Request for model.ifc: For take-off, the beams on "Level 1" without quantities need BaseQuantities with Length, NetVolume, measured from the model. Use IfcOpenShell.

First a look at what the model holds.

```python
import ifcopenshell
import ifcopenshell.util.element
import ifcopenshell.util.unit

model = ifcopenshell.open("model.ifc")
print(model.schema)
for unit_type in ("LENGTHUNIT", "AREAUNIT", "VOLUMEUNIT"):
    print(unit_type, ifcopenshell.util.unit.calculate_unit_scale(model, unit_type))
storey = next(s for s in model.by_type("IfcBuildingStorey") if s.Name == "Level 1")
beams = [e for e in ifcopenshell.util.element.get_decomposition(storey) if e.is_a("IfcBeam")]
for e in sorted(beams, key=lambda e: e.id()):
    print(e.id(), e.is_a(), e.Name, list(ifcopenshell.util.element.get_psets(e, qtos_only=True)), sep=" | ")
```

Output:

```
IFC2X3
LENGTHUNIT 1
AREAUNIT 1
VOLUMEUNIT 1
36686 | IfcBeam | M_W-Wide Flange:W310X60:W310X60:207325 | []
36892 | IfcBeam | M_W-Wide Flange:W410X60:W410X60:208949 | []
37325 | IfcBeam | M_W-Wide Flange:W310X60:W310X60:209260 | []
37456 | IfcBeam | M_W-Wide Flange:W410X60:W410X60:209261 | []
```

```python
import ifcopenshell
import ifcopenshell.api.pset
import ifcopenshell.geom
import ifcopenshell.util.element
import ifcopenshell.util.shape
import ifcopenshell.util.unit

model = ifcopenshell.open("model.ifc")
unit_scale = ifcopenshell.util.unit.calculate_unit_scale(model)
volume_scale = ifcopenshell.util.unit.calculate_unit_scale(model, "VOLUMEUNIT")
settings = ifcopenshell.geom.settings()

storey = next(s for s in model.by_type("IfcBuildingStorey") if s.Name == "Level 1")
beams = [e for e in ifcopenshell.util.element.get_decomposition(storey) if e.is_a("IfcBeam")]

for e in sorted(beams, key=lambda e: e.id()):
    if ifcopenshell.util.element.get_psets(e, qtos_only=True, should_inherit=False):
        continue
    # Geometry comes back in metres, in the element's own axes.
    shape = ifcopenshell.geom.create_shape(settings, e)
    values = {
        "Length": ifcopenshell.util.shape.get_max_xyz(shape.geometry) / unit_scale,
        "NetVolume": ifcopenshell.util.shape.get_volume(shape.geometry) / volume_scale,
    }
    qto = ifcopenshell.api.pset.add_qto(model, product=e, name="BaseQuantities")
    ifcopenshell.api.pset.edit_qto(model, qto=qto, properties=values)
    print(e.id(), {k: round(v, 3) for k, v in values.items()})

model.write("model_v2.ifc")
```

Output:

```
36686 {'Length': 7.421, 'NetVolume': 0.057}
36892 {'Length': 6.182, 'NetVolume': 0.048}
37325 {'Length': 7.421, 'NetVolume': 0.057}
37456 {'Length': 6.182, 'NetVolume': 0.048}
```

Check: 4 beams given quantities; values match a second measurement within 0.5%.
